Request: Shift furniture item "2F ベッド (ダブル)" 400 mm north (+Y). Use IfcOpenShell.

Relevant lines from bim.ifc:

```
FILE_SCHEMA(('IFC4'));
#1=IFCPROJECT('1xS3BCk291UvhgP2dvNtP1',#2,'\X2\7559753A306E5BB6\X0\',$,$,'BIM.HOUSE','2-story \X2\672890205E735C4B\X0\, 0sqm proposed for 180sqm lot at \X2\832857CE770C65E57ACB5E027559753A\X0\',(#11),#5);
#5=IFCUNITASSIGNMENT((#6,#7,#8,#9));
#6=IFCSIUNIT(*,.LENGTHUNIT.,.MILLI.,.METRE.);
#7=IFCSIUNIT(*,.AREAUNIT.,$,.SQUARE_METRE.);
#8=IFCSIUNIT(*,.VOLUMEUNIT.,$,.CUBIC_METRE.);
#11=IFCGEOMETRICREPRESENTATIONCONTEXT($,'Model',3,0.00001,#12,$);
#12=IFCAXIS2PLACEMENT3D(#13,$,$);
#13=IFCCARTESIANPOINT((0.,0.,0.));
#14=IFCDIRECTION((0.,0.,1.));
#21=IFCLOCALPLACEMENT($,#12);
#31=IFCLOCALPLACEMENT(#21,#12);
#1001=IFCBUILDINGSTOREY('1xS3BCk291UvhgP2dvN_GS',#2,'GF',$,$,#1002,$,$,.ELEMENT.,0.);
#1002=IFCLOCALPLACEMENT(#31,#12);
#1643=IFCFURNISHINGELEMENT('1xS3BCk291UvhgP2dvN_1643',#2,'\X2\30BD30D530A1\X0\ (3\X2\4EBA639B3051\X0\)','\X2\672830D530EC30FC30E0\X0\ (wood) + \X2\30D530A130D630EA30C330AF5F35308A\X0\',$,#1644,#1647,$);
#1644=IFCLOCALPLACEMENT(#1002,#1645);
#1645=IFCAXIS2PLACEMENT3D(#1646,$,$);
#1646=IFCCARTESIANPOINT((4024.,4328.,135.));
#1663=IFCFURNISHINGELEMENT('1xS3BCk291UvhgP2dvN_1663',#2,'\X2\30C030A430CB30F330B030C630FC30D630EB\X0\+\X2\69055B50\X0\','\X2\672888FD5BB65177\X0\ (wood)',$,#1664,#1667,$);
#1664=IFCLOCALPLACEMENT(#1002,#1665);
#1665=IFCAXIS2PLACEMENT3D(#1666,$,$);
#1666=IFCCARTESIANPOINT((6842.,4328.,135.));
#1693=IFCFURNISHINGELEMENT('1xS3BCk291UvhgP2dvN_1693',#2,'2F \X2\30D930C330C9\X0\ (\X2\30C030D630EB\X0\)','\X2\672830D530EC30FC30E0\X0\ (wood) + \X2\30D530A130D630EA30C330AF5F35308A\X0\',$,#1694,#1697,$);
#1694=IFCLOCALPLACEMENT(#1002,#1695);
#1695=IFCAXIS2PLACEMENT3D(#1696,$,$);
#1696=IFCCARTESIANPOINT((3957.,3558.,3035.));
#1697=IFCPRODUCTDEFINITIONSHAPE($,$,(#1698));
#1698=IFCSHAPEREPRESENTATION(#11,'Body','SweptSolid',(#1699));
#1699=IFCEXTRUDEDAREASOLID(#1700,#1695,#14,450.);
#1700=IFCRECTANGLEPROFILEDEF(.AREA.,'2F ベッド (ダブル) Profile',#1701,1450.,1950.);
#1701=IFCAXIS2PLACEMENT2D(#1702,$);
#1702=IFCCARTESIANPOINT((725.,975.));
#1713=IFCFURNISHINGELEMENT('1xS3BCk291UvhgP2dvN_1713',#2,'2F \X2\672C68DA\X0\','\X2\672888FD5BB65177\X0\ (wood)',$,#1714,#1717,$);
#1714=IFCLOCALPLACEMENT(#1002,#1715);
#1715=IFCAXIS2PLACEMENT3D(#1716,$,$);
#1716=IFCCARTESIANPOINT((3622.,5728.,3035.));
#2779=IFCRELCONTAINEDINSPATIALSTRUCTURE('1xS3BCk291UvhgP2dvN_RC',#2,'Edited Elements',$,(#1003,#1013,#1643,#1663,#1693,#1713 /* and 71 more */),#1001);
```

```python
import ifcopenshell
import ifcopenshell.api.geometry
import ifcopenshell.util.placement

model = ifcopenshell.open("bim.ifc")

item = model.by_id(1693)
matrix = ifcopenshell.util.placement.get_local_placement(item.ObjectPlacement)
matrix[1, 3] += 400.0
ifcopenshell.api.geometry.edit_object_placement(model, product=item, matrix=matrix, is_si=False)

print(ifcopenshell.util.placement.get_local_placement(item.ObjectPlacement).round(3) + 0.0)

model.write("bim_updated.ifc")
```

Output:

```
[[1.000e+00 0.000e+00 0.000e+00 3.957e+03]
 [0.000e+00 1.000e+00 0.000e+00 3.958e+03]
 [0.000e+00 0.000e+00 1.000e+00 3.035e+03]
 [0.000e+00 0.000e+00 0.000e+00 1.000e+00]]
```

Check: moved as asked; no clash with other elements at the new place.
